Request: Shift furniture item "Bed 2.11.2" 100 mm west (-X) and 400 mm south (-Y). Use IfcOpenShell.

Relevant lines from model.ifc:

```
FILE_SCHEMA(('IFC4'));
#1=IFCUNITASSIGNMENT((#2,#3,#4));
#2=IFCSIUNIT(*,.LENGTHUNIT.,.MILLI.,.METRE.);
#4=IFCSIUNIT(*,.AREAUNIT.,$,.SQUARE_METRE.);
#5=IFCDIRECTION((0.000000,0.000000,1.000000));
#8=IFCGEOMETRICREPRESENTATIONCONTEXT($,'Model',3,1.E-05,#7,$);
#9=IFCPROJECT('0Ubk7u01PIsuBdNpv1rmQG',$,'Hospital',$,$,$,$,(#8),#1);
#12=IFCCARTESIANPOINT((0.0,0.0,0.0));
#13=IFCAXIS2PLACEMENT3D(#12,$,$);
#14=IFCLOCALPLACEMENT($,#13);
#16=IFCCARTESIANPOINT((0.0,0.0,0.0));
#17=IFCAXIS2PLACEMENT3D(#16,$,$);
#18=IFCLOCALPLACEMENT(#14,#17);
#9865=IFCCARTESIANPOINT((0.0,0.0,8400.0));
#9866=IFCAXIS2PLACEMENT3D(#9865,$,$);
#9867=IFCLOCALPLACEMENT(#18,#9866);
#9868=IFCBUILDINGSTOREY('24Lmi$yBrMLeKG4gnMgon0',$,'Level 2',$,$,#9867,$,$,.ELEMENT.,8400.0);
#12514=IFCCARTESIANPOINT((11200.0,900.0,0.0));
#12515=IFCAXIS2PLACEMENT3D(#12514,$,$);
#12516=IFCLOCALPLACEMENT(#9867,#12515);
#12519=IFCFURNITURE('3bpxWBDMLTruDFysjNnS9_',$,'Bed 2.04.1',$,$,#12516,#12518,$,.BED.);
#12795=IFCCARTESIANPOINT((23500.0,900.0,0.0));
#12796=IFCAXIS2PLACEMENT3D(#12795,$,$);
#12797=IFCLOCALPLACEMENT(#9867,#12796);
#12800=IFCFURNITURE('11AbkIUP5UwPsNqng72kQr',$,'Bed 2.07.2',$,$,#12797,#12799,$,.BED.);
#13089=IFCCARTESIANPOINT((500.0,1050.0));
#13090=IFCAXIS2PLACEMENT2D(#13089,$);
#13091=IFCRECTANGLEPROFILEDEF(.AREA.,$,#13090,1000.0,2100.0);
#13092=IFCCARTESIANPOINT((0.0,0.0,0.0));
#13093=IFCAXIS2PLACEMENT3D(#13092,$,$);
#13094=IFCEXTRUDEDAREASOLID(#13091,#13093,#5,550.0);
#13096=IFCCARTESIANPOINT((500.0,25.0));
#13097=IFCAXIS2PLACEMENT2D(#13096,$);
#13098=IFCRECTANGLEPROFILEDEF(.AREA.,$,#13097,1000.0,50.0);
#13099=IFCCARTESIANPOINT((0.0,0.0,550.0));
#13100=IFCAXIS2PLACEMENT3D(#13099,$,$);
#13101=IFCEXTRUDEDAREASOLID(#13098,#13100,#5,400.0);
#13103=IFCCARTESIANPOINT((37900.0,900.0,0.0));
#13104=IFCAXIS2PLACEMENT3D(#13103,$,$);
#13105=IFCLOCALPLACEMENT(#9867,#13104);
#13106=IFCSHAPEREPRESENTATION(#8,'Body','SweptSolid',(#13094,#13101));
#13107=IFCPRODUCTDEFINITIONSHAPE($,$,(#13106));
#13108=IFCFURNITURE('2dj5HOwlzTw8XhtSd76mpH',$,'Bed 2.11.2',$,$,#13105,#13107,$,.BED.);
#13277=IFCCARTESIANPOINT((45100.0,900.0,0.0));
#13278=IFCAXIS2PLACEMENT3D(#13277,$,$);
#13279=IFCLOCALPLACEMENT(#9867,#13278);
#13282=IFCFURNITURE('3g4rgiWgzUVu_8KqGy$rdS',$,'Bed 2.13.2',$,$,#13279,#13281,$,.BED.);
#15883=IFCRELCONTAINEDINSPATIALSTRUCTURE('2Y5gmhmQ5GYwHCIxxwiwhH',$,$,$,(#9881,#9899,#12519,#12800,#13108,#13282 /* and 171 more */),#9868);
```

```python
import ifcopenshell
import ifcopenshell.api.geometry
import ifcopenshell.util.placement
import ifcopenshell.util.unit

model = ifcopenshell.open("model.ifc")
unit_scale = ifcopenshell.util.unit.calculate_unit_scale(model)

item = model.by_id(13108)
matrix = ifcopenshell.util.placement.get_local_placement(item.ObjectPlacement)
matrix[0, 3] -= 0.1 / unit_scale
matrix[1, 3] -= 0.4 / unit_scale
ifcopenshell.api.geometry.edit_object_placement(model, product=item, matrix=matrix, is_si=False)

print(ifcopenshell.util.placement.get_local_placement(item.ObjectPlacement).round(3) + 0.0)

model.write("model_v2.ifc")
```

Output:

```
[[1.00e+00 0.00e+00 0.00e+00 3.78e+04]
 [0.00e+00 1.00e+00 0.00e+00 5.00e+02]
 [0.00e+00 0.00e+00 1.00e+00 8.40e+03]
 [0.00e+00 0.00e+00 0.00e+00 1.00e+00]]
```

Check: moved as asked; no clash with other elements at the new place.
